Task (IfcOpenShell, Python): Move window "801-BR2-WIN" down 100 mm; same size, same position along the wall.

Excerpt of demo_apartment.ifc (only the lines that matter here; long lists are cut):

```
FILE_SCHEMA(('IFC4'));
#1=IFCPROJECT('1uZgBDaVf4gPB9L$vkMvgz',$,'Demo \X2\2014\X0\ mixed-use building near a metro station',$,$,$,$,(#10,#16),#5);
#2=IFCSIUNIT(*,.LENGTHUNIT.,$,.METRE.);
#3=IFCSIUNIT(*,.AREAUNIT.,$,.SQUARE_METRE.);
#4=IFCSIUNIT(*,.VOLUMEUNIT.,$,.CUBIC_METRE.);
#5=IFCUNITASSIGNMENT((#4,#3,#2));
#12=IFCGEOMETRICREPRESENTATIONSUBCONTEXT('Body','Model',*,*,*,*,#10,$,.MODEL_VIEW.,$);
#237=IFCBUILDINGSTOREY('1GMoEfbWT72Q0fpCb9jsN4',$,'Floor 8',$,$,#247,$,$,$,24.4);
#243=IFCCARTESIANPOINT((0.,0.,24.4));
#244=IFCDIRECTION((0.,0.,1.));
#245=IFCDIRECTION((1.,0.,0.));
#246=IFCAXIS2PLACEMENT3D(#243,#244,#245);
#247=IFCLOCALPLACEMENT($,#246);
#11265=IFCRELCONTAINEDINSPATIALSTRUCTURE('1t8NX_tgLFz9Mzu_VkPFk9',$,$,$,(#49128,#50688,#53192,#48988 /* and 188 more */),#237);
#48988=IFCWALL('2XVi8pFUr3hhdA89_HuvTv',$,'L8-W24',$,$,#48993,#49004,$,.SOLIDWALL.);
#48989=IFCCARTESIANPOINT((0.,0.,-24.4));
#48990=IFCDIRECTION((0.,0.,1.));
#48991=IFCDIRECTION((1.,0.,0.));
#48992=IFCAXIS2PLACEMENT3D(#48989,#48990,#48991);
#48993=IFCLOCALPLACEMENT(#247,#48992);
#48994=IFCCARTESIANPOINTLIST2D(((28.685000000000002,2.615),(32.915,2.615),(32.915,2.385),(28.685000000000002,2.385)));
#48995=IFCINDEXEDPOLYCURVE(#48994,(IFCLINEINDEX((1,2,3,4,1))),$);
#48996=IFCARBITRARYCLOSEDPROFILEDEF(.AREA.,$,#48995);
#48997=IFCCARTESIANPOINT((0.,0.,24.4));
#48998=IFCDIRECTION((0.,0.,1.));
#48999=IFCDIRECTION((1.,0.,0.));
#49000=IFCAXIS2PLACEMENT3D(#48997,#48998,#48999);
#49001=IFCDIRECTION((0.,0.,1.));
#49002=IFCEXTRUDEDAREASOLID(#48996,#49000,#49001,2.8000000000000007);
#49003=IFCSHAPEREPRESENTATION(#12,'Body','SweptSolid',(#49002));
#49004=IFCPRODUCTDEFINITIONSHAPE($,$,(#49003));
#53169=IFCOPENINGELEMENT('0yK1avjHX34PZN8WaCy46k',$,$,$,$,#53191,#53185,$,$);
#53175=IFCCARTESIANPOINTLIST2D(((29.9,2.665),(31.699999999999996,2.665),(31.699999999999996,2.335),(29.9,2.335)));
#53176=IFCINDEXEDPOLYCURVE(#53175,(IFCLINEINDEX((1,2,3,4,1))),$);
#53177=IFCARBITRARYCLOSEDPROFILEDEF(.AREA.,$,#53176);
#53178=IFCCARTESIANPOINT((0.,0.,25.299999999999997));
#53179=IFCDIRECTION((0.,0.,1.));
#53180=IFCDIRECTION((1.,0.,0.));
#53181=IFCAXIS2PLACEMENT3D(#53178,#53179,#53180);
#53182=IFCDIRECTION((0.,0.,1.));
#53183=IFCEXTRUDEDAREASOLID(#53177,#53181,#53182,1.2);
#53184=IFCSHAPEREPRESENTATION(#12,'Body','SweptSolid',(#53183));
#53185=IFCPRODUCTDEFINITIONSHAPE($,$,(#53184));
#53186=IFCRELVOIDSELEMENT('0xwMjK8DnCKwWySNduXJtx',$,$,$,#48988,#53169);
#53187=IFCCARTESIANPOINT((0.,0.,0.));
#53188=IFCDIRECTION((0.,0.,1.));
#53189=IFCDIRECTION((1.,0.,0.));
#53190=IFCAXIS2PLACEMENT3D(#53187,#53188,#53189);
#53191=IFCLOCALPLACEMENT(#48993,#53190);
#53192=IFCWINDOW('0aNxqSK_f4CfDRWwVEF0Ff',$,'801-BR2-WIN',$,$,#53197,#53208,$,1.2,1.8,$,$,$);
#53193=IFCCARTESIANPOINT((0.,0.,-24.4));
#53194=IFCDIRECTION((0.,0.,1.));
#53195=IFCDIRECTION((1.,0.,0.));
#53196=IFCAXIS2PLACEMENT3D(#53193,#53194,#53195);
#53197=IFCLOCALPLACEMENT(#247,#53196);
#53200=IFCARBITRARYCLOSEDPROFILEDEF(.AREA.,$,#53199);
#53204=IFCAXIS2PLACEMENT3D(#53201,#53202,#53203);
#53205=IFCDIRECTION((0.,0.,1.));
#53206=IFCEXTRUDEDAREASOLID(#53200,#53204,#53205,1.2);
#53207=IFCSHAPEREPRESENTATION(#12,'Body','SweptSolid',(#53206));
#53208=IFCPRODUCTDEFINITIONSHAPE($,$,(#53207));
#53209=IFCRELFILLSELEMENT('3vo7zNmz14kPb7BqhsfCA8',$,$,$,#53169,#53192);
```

```python
import numpy as np
import ifcopenshell
import ifcopenshell.api.geometry
import ifcopenshell.util.placement
import ifcopenshell.util.unit

model = ifcopenshell.open("demo_apartment.ifc")
unit_scale = ifcopenshell.util.unit.calculate_unit_scale(model)

window = model.by_guid("0aNxqSK_f4CfDRWwVEF0Ff")
opening = window.FillsVoids[0].RelatingOpeningElement
dz = -0.1

shift = np.array([0.0, 0.0, dz])
# The window is not placed relative to its opening, so move both.
for product in (opening, window):
    matrix = ifcopenshell.util.placement.get_local_placement(product.ObjectPlacement)
    matrix[:3, 3] += shift
    ifcopenshell.api.geometry.edit_object_placement(model, product=product, matrix=matrix, is_si=False)

print(f"moved by {dz * unit_scale:+.3f} m")

model.write("demo_apartment_v2.ifc")
```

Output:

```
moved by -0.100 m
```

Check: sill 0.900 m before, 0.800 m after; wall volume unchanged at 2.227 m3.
